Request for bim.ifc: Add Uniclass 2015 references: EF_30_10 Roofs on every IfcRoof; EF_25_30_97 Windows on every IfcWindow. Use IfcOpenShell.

First a look at what the model holds.

```python
import ifcopenshell

model = ifcopenshell.open("bim.ifc")
print(model.schema)
print("classifications:", [c.Name for c in model.by_type("IfcClassification")])
for ifc_class in ("IfcDoor", "IfcRoof", "IfcStair", "IfcWall", "IfcWindow"):
    print(ifc_class, len(model.by_type(ifc_class)))
```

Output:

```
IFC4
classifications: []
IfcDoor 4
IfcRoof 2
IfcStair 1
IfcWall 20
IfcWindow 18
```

```python
import ifcopenshell
import ifcopenshell.api.classification

model = ifcopenshell.open("bim.ifc")

system = ifcopenshell.api.classification.add_classification(model, classification="Uniclass 2015")

codes = {
    "IfcRoof": ("EF_30_10", "Roofs"),
    "IfcWindow": ("EF_25_30_97", "Windows"),
}
for ifc_class, (code, name) in codes.items():
    products = model.by_type(ifc_class)
    ifcopenshell.api.classification.add_reference(
        model, products=products, classification=system, identification=code, name=name
    )
    print(code, len(products))

model.write("bim_updated.ifc")
```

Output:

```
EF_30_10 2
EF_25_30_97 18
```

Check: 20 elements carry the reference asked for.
